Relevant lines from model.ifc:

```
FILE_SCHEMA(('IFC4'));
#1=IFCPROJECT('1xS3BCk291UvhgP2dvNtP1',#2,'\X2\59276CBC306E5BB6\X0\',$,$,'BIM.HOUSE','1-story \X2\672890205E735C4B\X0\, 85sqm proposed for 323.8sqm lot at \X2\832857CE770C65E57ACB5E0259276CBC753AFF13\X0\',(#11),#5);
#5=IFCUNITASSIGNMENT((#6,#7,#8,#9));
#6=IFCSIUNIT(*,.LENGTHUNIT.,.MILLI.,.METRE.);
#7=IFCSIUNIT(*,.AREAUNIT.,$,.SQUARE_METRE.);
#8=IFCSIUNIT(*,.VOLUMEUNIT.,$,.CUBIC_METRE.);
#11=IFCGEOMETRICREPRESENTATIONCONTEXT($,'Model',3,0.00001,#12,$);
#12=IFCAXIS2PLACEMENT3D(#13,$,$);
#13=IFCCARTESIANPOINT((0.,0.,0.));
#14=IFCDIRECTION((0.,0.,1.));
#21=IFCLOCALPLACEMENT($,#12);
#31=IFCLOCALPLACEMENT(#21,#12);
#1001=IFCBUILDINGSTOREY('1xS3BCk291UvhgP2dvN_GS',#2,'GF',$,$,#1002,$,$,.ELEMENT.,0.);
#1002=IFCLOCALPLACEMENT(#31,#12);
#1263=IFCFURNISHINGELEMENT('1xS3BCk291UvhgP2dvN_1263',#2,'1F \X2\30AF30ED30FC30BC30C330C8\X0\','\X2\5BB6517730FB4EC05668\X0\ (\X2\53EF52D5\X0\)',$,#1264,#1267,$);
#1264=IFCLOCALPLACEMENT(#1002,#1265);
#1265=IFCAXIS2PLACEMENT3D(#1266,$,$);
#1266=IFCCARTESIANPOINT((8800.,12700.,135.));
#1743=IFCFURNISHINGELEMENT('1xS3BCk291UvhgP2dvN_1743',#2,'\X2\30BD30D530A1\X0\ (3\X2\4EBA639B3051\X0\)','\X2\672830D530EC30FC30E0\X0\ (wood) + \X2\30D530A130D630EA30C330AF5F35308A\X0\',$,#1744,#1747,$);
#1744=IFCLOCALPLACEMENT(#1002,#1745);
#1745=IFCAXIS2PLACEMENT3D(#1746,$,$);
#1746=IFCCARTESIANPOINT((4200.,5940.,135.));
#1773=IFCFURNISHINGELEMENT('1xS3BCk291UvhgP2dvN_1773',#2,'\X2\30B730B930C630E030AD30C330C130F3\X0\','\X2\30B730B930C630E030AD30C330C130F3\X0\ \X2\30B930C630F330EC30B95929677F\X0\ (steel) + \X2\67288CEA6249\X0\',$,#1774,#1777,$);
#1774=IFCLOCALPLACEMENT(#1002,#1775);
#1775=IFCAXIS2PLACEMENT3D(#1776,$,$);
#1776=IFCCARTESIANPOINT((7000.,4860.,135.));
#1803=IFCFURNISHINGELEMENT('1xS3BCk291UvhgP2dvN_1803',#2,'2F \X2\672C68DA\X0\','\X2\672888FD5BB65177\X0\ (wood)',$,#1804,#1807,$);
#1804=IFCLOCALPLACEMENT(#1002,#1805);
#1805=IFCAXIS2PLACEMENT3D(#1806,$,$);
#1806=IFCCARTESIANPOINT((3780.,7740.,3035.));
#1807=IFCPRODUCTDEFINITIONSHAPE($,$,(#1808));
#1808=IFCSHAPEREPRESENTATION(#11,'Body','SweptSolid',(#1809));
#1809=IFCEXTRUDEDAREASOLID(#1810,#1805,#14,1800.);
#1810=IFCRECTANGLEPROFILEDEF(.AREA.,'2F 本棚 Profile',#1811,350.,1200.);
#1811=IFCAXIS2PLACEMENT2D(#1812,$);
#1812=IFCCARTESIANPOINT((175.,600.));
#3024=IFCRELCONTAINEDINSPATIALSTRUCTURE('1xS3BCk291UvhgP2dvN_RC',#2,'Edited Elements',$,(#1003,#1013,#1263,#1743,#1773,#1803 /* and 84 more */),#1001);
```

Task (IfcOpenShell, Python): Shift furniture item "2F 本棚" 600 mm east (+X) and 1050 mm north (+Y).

```python
import ifcopenshell
import ifcopenshell.api.geometry
import ifcopenshell.util.placement
import ifcopenshell.util.unit

model = ifcopenshell.open("model.ifc")
unit_scale = ifcopenshell.util.unit.calculate_unit_scale(model)

item = model.by_guid("1xS3BCk291UvhgP2dvN_1803")
matrix = ifcopenshell.util.placement.get_local_placement(item.ObjectPlacement)
matrix[0, 3] += 0.6 / unit_scale
matrix[1, 3] += 1.05 / unit_scale
ifcopenshell.api.geometry.edit_object_placement(model, product=item, matrix=matrix, is_si=False)

print(ifcopenshell.util.placement.get_local_placement(item.ObjectPlacement).round(3) + 0.0)

model.write("model_rev.ifc")
```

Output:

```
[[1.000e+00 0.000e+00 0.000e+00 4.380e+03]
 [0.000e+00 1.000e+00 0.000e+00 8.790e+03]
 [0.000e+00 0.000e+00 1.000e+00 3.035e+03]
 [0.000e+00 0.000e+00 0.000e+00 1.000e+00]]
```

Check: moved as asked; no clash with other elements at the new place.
